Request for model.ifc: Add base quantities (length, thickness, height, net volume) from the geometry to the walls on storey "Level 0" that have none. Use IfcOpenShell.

First a look at what the model holds.

```python
import ifcopenshell
import ifcopenshell.util.element
import ifcopenshell.util.unit

model = ifcopenshell.open("model.ifc")
print(model.schema)
for unit_type in ("LENGTHUNIT", "AREAUNIT", "VOLUMEUNIT"):
    print(unit_type, ifcopenshell.util.unit.calculate_unit_scale(model, unit_type))
storey = next(s for s in model.by_type("IfcBuildingStorey") if s.Name == "Level 0")
walls = [e for e in ifcopenshell.util.element.get_decomposition(storey) if e.is_a("IfcWall")]
for e in sorted(walls, key=lambda e: e.id()):
    print(e.id(), e.is_a(), e.Name, list(ifcopenshell.util.element.get_psets(e, qtos_only=True)), sep=" | ")
```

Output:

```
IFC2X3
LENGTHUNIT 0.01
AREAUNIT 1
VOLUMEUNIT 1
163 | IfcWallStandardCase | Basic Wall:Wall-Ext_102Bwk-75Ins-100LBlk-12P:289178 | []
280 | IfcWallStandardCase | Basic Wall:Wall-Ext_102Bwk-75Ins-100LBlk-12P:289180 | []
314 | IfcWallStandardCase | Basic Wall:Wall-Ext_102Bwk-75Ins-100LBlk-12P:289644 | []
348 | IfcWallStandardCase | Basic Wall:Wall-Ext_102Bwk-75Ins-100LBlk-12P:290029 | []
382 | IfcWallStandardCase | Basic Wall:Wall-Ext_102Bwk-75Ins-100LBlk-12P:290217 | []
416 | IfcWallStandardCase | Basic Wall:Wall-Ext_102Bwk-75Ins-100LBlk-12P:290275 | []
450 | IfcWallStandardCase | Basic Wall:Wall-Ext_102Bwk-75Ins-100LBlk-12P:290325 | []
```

```python
import ifcopenshell
import ifcopenshell.api.pset
import ifcopenshell.geom
import ifcopenshell.util.element
import ifcopenshell.util.shape
import ifcopenshell.util.unit

model = ifcopenshell.open("model.ifc")
unit_scale = ifcopenshell.util.unit.calculate_unit_scale(model)
volume_scale = ifcopenshell.util.unit.calculate_unit_scale(model, "VOLUMEUNIT")
settings = ifcopenshell.geom.settings()

storey = next(s for s in model.by_type("IfcBuildingStorey") if s.Name == "Level 0")
walls = [e for e in ifcopenshell.util.element.get_decomposition(storey) if e.is_a("IfcWall")]

for e in sorted(walls, key=lambda e: e.id()):
    if ifcopenshell.util.element.get_psets(e, qtos_only=True, should_inherit=False):
        continue
    # Geometry comes back in metres, in the element's own axes.
    shape = ifcopenshell.geom.create_shape(settings, e)
    values = {
        "Length": ifcopenshell.util.shape.get_x(shape.geometry) / unit_scale,
        "Width": ifcopenshell.util.shape.get_y(shape.geometry) / unit_scale,
        "Height": ifcopenshell.util.shape.get_z(shape.geometry) / unit_scale,
        "NetVolume": ifcopenshell.util.shape.get_volume(shape.geometry) / volume_scale,
    }
    qto = ifcopenshell.api.pset.add_qto(model, product=e, name="BaseQuantities")
    ifcopenshell.api.pset.edit_qto(model, qto=qto, properties=values)
    print(e.id(), {k: round(v, 3) for k, v in values.items()})

model.write("model_rev.ifc")
```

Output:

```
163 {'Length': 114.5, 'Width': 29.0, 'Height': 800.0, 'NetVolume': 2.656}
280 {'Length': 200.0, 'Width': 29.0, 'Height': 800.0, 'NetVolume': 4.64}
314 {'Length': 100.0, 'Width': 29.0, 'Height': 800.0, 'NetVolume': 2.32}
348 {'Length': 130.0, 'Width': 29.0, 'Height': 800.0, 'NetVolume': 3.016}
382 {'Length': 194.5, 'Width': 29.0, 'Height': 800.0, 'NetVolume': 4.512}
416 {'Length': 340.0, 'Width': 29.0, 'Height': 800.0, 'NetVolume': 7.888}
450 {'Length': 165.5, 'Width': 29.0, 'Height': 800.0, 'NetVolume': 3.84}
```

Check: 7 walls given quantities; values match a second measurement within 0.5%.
